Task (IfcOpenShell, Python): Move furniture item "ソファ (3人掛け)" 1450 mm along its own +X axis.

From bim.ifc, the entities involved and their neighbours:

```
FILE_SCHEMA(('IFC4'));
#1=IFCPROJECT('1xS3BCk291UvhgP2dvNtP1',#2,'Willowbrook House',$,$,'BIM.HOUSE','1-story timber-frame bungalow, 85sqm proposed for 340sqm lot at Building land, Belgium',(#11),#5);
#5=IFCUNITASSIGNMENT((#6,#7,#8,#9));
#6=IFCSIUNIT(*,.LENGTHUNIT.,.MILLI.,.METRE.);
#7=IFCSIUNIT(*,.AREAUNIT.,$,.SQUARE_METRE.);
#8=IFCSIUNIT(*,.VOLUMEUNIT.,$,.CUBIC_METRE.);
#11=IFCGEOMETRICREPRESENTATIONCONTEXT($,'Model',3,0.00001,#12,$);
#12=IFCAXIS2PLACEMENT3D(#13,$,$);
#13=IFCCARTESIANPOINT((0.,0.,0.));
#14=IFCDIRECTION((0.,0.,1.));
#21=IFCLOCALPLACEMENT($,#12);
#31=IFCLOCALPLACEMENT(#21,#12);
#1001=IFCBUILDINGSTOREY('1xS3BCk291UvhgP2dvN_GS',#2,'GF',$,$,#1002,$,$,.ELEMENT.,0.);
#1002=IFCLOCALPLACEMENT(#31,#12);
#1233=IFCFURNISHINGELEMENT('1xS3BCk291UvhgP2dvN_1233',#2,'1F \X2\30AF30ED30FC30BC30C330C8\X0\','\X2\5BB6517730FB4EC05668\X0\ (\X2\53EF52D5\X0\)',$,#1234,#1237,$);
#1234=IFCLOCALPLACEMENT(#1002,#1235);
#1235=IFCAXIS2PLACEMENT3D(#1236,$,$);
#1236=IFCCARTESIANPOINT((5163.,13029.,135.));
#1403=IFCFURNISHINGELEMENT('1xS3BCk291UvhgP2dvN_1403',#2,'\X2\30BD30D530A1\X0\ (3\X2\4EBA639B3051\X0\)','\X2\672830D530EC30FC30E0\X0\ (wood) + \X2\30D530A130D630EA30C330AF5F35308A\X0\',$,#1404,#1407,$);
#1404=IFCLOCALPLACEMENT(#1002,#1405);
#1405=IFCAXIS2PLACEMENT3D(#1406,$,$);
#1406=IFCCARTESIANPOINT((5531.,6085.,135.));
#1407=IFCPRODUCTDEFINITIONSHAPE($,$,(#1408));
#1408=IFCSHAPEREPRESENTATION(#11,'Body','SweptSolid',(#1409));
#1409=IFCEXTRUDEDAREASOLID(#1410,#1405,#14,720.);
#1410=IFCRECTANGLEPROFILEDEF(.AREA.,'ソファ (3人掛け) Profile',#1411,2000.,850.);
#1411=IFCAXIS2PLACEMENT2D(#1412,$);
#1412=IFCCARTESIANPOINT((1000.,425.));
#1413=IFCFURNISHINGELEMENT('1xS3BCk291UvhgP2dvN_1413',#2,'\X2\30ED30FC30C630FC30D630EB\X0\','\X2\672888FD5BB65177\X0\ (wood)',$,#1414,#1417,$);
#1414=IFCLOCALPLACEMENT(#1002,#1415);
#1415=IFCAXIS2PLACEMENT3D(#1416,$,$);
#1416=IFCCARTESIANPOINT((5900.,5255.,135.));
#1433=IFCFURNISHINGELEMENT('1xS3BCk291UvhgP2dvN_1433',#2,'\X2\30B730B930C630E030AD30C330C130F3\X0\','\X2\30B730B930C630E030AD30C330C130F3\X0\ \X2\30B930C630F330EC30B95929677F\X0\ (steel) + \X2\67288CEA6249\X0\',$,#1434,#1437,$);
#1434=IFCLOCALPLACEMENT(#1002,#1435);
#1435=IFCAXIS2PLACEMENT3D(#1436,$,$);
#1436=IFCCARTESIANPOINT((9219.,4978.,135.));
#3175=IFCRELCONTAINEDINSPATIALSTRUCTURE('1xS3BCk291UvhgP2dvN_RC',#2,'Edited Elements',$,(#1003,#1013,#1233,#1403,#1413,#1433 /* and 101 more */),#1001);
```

```python
import ifcopenshell
import ifcopenshell.api.geometry
import ifcopenshell.util.placement

model = ifcopenshell.open("bim.ifc")

item = model.by_guid("1xS3BCk291UvhgP2dvN_1403")
matrix = ifcopenshell.util.placement.get_local_placement(item.ObjectPlacement)
matrix[:3, 3] += matrix[:3, 0] * 1450.0
ifcopenshell.api.geometry.edit_object_placement(model, product=item, matrix=matrix, is_si=False)

print(ifcopenshell.util.placement.get_local_placement(item.ObjectPlacement).round(3) + 0.0)

model.write("bim_edited.ifc")
```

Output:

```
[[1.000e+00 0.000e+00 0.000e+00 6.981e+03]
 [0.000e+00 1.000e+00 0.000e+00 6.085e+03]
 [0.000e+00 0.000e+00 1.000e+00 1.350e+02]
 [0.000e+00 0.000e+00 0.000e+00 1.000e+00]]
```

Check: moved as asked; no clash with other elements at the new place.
